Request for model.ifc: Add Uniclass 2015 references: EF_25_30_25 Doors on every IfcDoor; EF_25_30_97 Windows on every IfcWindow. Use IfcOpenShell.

First a look at what the model holds.

```python
import ifcopenshell

model = ifcopenshell.open("model.ifc")
print(model.schema)
print("classifications:", [c.Name for c in model.by_type("IfcClassification")])
for ifc_class in ("IfcDoor", "IfcRoof", "IfcStair", "IfcWall", "IfcWindow"):
    print(ifc_class, len(model.by_type(ifc_class)))
```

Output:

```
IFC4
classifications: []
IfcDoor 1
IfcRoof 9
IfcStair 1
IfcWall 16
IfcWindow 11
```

```python
import ifcopenshell
import ifcopenshell.api.classification

model = ifcopenshell.open("model.ifc")

system = ifcopenshell.api.classification.add_classification(model, classification="Uniclass 2015")

codes = {
    "IfcDoor": ("EF_25_30_25", "Doors"),
    "IfcWindow": ("EF_25_30_97", "Windows"),
}
for ifc_class, (code, name) in codes.items():
    products = model.by_type(ifc_class)
    ifcopenshell.api.classification.add_reference(
        model, products=products, classification=system, identification=code, name=name
    )
    print(code, len(products))

model.write("model_updated.ifc")
```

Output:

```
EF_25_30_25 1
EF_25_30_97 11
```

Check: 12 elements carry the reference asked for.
